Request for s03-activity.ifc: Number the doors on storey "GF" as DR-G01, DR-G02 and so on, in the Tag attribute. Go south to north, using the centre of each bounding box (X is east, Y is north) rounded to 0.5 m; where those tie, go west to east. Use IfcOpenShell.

First a look at what the model holds.

```python
import ifcopenshell
import ifcopenshell.util.element
import ifcopenshell.util.placement

model = ifcopenshell.open("s03-activity.ifc")
print(model.schema)
storey = next(s for s in model.by_type("IfcBuildingStorey") if s.Name == "GF")
doors = [e for e in ifcopenshell.util.element.get_decomposition(storey) if e.is_a("IfcDoor")]
for e in sorted(doors, key=lambda e: e.id()):
    origin = ifcopenshell.util.placement.get_local_placement(e.ObjectPlacement)[:3, 3]
    print(e.id(), e.Tag, e.Name, origin.round(2) + 0.0, sep=" | ")
```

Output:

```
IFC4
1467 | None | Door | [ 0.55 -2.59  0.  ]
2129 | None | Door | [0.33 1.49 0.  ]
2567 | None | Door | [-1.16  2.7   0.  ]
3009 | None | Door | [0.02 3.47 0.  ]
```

```python
import ifcopenshell
import ifcopenshell.geom
import ifcopenshell.util.element
import ifcopenshell.util.shape

model = ifcopenshell.open("s03-activity.ifc")
settings = ifcopenshell.geom.settings()
settings.set("use-world-coords", True)


def centre(element):
    shape = ifcopenshell.geom.create_shape(settings, element)
    return ifcopenshell.util.shape.get_bbox_centroid(shape.geometry)


storey = next(s for s in model.by_type("IfcBuildingStorey") if s.Name == "GF")
doors = [e for e in ifcopenshell.util.element.get_decomposition(storey) if e.is_a("IfcDoor")]

# Insertion points can sit at a corner or the storey origin, so sort by the geometry (in metres).
centres = {e: centre(e) for e in doors}
doors.sort(key=lambda e: (round(centres[e][1] / 0.5), centres[e][0]))

for i, e in enumerate(doors, start=1):
    number = f"DR-G{i:02d}"
    e.Tag = number
    print(e.id(), number)

model.write("s03-activity_v2.ifc")
```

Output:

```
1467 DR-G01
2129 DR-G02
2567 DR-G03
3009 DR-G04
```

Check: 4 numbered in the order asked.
